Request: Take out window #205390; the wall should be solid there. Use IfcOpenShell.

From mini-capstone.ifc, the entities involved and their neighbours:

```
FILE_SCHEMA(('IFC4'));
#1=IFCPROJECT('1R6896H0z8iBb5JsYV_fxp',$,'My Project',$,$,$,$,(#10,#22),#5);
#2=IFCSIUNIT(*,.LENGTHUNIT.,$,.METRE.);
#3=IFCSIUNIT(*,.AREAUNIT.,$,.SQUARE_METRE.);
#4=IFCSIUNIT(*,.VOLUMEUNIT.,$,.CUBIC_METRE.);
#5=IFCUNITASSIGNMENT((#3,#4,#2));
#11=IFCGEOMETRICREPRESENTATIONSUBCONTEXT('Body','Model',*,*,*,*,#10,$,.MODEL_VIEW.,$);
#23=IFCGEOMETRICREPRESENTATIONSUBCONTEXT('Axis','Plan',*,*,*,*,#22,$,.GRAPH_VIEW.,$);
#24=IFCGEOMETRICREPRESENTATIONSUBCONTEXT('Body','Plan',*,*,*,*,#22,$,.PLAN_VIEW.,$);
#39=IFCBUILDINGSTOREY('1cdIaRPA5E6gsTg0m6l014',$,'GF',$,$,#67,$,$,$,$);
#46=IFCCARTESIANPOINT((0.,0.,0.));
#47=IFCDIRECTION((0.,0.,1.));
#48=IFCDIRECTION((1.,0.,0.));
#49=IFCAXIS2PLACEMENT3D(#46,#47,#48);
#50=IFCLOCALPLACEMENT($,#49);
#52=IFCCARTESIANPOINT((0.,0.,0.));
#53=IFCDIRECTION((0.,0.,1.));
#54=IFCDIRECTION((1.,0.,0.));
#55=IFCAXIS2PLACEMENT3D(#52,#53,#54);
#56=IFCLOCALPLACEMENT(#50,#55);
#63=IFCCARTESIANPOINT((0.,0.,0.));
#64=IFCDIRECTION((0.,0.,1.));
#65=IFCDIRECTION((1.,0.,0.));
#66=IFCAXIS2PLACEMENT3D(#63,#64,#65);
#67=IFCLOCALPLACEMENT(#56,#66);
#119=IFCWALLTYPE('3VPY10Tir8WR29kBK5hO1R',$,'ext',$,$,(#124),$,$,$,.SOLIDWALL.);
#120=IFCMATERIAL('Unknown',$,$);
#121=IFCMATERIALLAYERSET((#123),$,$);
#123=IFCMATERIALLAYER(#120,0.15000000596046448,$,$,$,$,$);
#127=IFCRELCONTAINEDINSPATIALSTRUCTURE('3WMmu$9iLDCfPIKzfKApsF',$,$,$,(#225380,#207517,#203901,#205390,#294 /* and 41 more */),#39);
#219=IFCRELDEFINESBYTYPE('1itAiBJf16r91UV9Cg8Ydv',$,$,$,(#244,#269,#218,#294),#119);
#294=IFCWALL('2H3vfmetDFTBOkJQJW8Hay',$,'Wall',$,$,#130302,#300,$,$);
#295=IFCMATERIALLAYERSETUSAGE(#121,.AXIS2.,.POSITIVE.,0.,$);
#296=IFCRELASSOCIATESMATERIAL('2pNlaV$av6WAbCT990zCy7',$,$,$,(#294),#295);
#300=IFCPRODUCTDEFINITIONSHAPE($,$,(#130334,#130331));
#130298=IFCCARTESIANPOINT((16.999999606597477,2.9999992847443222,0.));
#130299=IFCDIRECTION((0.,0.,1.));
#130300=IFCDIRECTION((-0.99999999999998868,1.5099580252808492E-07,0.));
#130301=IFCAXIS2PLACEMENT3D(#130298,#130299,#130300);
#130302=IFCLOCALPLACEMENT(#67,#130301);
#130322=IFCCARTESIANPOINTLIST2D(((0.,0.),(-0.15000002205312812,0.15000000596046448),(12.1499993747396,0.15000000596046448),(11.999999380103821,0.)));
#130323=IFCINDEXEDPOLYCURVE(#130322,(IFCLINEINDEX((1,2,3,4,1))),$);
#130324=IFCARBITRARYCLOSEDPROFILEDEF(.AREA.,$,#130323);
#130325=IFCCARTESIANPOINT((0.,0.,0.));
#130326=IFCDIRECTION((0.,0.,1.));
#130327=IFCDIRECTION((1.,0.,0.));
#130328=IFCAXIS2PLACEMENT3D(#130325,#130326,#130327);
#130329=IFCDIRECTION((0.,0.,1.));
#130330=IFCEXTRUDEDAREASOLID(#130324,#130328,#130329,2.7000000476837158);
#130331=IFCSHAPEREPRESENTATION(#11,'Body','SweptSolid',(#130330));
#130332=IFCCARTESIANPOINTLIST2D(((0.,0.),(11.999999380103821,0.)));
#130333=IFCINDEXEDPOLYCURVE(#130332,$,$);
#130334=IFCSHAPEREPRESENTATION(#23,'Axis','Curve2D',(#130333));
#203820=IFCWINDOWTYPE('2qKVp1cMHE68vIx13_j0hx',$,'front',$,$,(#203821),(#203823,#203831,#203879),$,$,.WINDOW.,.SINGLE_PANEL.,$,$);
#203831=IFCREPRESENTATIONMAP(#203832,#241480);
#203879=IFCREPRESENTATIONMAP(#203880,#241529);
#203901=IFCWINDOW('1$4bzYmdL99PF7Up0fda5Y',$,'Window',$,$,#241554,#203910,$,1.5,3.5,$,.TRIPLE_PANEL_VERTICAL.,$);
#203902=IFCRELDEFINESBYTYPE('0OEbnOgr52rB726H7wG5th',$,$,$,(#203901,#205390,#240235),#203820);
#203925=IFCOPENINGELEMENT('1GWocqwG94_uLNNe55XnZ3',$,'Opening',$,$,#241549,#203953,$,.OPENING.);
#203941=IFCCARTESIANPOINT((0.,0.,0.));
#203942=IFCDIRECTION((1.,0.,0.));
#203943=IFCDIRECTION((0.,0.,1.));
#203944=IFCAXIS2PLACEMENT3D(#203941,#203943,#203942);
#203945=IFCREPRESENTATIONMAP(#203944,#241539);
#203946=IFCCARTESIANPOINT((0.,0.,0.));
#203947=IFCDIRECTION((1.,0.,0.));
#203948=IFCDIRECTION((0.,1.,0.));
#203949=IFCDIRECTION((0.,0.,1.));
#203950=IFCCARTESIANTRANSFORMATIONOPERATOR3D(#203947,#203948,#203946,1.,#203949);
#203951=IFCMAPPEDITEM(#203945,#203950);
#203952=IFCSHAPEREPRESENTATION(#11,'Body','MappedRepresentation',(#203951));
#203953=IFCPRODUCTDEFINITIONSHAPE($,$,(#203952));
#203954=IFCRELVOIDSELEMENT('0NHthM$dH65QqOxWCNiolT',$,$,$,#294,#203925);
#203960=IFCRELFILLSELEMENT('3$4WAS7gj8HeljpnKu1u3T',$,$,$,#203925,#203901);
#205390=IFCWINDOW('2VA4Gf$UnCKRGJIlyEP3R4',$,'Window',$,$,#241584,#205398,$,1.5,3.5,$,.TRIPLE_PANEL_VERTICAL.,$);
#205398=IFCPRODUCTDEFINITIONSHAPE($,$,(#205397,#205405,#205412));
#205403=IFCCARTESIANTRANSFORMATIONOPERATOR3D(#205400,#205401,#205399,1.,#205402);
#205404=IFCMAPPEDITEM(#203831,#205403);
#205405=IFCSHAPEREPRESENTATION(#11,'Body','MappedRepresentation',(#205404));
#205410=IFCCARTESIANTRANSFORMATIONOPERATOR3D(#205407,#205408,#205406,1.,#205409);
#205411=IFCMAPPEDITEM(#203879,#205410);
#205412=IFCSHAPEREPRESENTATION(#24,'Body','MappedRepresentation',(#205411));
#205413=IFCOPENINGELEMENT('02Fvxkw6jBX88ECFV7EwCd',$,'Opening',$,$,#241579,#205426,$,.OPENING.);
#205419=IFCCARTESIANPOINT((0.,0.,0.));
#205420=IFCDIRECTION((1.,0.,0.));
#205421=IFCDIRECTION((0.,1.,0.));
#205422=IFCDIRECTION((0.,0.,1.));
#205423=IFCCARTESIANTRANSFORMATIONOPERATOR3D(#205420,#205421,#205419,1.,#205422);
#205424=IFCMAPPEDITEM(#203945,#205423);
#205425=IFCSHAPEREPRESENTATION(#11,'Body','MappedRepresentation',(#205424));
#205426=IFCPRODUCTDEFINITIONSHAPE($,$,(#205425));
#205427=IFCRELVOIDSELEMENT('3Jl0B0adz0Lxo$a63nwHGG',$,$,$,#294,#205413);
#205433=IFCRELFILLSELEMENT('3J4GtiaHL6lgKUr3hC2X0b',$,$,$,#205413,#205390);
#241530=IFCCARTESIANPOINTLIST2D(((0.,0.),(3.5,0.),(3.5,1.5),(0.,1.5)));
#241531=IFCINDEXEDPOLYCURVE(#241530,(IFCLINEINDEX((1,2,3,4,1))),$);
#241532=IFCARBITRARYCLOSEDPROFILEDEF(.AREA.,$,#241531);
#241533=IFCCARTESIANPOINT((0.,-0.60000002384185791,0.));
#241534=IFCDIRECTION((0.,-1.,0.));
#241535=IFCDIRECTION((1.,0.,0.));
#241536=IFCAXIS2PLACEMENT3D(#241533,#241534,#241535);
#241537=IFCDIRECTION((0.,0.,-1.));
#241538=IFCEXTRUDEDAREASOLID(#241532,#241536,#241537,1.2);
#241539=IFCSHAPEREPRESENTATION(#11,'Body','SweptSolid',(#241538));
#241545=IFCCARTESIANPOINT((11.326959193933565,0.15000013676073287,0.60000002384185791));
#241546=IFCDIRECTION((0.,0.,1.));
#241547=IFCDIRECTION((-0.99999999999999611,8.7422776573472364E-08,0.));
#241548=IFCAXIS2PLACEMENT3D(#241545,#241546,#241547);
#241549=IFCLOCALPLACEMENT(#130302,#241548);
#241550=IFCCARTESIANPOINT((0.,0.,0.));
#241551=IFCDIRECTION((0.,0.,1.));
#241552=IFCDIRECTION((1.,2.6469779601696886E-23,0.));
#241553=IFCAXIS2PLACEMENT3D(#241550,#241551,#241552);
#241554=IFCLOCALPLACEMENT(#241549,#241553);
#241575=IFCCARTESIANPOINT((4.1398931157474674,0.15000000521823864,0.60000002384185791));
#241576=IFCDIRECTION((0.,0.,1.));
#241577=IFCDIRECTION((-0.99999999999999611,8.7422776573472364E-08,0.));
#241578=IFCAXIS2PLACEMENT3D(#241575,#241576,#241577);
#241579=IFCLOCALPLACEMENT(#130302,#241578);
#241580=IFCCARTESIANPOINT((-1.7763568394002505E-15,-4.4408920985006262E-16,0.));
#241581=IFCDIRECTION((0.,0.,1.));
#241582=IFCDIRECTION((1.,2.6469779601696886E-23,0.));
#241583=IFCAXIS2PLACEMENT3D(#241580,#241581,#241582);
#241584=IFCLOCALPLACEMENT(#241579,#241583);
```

```python
import ifcopenshell
import ifcopenshell.api.feature
import ifcopenshell.api.root
import ifcopenshell.geom
import ifcopenshell.util.shape

model = ifcopenshell.open("mini-capstone.ifc")
settings = ifcopenshell.geom.settings()


def volume(element):
    """Net volume in cubic metres, openings subtracted."""
    shape = ifcopenshell.geom.create_shape(settings, element)
    return ifcopenshell.util.shape.get_volume(shape.geometry)


window = model.by_guid("2VA4Gf$UnCKRGJIlyEP3R4")
opening = window.FillsVoids[0].RelatingOpeningElement
wall = opening.VoidsElements[0].RelatingBuildingElement
before = volume(wall)

ifcopenshell.api.root.remove_product(model, product=window)
ifcopenshell.api.feature.remove_feature(model, feature=opening)

after = volume(wall)

print(f"wall volume {before:.3f} -> {after:.3f} m3")

model.write("mini-capstone_edited.ifc")
```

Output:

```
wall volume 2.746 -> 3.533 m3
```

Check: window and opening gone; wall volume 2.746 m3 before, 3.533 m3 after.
